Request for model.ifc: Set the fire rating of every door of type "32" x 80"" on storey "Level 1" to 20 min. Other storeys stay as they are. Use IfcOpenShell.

First a look at what the model holds.

```python
import ifcopenshell
import ifcopenshell.util.element

model = ifcopenshell.open("model.ifc")
print(model.schema)
storey = next(s for s in model.by_type("IfcBuildingStorey") if s.Name == "Level 1")
doors = [e for e in ifcopenshell.util.element.get_decomposition(storey) if e.is_a("IfcDoor")]
seen = {}
for e in doors:
    element_type = ifcopenshell.util.element.get_type(e)
    key = (element_type.Name if element_type != e and element_type else None, ifcopenshell.util.element.get_pset(e, "Pset_DoorCommon", "FireRating"))
    seen[key] = seen.get(key, 0) + 1
for (name, value), count in sorted(seen.items(), key=str):
    print(count, "x", name, "|", value)
```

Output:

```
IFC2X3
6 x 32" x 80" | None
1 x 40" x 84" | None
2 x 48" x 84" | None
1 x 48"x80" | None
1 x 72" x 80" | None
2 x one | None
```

```python
import ifcopenshell
import ifcopenshell.api.pset
import ifcopenshell.util.element

model = ifcopenshell.open("model.ifc")

storey = next(s for s in model.by_type("IfcBuildingStorey") if s.Name == "Level 1")
doors = [e for e in ifcopenshell.util.element.get_decomposition(storey) if e.is_a("IfcDoor")]

count = 0
for e in doors:
    element_type = ifcopenshell.util.element.get_type(e)
    if element_type in (None, e) or element_type.Name != '32" x 80"':
        continue
    # add_pset returns the element's existing set when there is one.
    pset = ifcopenshell.api.pset.add_pset(model, product=e, name="Pset_DoorCommon")
    ifcopenshell.api.pset.edit_pset(model, pset=pset, properties={"FireRating": "20 min"})
    count += 1

print(count, "doors updated")

model.write("model_v2.ifc")
```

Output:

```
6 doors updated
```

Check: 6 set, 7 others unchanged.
